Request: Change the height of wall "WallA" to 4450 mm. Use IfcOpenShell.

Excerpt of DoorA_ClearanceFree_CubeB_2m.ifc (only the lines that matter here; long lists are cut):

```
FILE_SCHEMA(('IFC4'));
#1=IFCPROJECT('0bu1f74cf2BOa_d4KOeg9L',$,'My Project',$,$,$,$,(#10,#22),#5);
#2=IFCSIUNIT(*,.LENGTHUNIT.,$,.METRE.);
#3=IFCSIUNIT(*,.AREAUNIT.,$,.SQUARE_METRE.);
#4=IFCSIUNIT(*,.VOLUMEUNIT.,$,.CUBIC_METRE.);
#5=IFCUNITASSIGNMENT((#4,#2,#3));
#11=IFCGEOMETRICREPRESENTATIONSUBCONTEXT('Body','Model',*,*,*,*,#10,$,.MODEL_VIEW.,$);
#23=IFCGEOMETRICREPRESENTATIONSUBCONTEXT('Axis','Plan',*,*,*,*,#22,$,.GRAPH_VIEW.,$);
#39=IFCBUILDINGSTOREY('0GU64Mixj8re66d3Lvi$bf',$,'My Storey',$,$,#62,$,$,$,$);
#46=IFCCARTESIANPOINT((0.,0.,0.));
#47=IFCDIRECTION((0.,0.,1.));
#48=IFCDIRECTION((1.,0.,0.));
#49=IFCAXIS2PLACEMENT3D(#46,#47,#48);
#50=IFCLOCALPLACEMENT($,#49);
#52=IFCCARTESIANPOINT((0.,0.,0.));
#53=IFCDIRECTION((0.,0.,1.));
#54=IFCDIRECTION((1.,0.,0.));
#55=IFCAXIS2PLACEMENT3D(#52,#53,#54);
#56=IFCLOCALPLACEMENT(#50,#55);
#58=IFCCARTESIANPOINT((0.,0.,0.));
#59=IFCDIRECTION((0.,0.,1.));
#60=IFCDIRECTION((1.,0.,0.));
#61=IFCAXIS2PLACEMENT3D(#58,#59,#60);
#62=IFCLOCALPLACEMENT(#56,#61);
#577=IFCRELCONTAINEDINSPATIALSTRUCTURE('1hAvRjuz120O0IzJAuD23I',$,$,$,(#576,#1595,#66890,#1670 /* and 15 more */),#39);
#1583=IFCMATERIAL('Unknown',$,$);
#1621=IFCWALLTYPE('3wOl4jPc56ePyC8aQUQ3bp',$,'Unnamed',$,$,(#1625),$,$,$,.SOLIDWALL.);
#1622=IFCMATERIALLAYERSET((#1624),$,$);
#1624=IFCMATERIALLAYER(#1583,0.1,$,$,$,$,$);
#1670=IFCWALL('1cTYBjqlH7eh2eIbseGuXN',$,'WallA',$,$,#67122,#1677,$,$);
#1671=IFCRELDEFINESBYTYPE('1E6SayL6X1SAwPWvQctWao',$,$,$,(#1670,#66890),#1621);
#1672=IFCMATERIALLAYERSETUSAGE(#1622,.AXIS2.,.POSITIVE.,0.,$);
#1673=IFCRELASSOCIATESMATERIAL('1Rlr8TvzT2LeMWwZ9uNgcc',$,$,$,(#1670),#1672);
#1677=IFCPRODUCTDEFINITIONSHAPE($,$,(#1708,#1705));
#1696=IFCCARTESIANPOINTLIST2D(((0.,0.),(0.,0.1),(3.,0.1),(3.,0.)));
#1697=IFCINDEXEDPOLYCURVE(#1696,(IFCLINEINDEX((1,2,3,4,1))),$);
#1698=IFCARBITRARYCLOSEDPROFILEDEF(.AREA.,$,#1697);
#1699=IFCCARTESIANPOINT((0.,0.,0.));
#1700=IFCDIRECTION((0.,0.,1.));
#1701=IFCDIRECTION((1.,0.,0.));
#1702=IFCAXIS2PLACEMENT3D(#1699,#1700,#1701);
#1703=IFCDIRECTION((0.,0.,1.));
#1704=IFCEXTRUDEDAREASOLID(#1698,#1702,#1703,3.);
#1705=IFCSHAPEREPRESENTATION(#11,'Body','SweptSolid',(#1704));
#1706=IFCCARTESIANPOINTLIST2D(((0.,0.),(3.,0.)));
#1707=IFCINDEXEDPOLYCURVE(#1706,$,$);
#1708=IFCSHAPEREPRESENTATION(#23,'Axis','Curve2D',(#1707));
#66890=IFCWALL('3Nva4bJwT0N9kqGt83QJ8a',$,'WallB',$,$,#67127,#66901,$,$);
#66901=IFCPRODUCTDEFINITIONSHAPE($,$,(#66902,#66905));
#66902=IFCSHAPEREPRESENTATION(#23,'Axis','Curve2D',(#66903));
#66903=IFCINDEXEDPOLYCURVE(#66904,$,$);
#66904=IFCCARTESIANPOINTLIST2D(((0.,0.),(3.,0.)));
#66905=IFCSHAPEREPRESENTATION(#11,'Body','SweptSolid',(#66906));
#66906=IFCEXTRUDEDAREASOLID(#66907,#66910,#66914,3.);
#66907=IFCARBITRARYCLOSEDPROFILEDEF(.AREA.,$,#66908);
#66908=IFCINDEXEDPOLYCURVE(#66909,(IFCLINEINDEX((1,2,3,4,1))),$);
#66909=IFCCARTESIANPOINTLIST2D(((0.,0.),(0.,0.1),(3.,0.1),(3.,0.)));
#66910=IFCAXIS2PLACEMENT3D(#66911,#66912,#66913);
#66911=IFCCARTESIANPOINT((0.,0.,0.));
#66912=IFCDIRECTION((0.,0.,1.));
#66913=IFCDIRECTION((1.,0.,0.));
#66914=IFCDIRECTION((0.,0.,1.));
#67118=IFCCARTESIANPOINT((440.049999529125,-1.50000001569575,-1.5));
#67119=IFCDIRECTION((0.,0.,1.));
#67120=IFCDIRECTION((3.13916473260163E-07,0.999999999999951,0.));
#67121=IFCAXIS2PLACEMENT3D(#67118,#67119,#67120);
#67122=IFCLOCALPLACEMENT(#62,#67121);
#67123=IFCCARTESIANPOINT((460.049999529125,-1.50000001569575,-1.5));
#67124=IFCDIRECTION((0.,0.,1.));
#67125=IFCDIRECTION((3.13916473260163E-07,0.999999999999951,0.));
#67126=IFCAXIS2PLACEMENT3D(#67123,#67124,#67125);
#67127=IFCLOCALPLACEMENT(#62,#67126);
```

```python
import ifcopenshell
import ifcopenshell.geom
import ifcopenshell.util.representation
import ifcopenshell.util.shape

model = ifcopenshell.open("DoorA_ClearanceFree_CubeB_2m.ifc")
settings = ifcopenshell.geom.settings()


def volume(element):
    """Net volume in cubic metres, openings subtracted."""
    shape = ifcopenshell.geom.create_shape(settings, element)
    return ifcopenshell.util.shape.get_volume(shape.geometry)


wall = model.by_id(1670)
before = volume(wall)

body = ifcopenshell.util.representation.get_representation(wall, "Model", "Body")
solid = body.Items[0]
old_height = solid.Depth
solid.Depth = 4.45
after = volume(wall)

print(f"height {old_height:g} -> {solid.Depth:g}, volume {before:.3f} -> {after:.3f} m3")

model.write("DoorA_ClearanceFree_CubeB_2m_v2.ifc")
```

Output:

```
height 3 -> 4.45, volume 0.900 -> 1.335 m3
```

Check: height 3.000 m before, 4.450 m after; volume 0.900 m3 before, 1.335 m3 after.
